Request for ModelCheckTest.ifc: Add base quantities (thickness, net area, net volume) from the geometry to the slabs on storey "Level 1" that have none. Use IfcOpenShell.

First a look at what the model holds.

```python
import ifcopenshell
import ifcopenshell.util.element
import ifcopenshell.util.unit

model = ifcopenshell.open("ModelCheckTest.ifc")
print(model.schema)
for unit_type in ("LENGTHUNIT", "AREAUNIT", "VOLUMEUNIT"):
    print(unit_type, ifcopenshell.util.unit.calculate_unit_scale(model, unit_type))
storey = next(s for s in model.by_type("IfcBuildingStorey") if s.Name == "Level 1")
slabs = [e for e in ifcopenshell.util.element.get_decomposition(storey) if e.is_a("IfcSlab")]
for e in sorted(slabs, key=lambda e: e.id()):
    print(e.id(), e.is_a(), e.Name, list(ifcopenshell.util.element.get_psets(e, qtos_only=True)), sep=" | ")
```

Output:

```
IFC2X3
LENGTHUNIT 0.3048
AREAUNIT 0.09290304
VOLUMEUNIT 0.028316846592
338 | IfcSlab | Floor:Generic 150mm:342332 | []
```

```python
import ifcopenshell
import ifcopenshell.api.pset
import ifcopenshell.geom
import ifcopenshell.util.element
import ifcopenshell.util.shape
import ifcopenshell.util.unit

model = ifcopenshell.open("ModelCheckTest.ifc")
unit_scale = ifcopenshell.util.unit.calculate_unit_scale(model)
area_scale = ifcopenshell.util.unit.calculate_unit_scale(model, "AREAUNIT")
volume_scale = ifcopenshell.util.unit.calculate_unit_scale(model, "VOLUMEUNIT")
settings = ifcopenshell.geom.settings()

storey = next(s for s in model.by_type("IfcBuildingStorey") if s.Name == "Level 1")
slabs = [e for e in ifcopenshell.util.element.get_decomposition(storey) if e.is_a("IfcSlab")]

for e in sorted(slabs, key=lambda e: e.id()):
    if ifcopenshell.util.element.get_psets(e, qtos_only=True, should_inherit=False):
        continue
    # Geometry comes back in metres, in the element's own axes.
    shape = ifcopenshell.geom.create_shape(settings, e)
    values = {
        "Width": ifcopenshell.util.shape.get_z(shape.geometry) / unit_scale,
        "NetArea": ifcopenshell.util.shape.get_footprint_area(shape.geometry) / area_scale,
        "NetVolume": ifcopenshell.util.shape.get_volume(shape.geometry) / volume_scale,
    }
    qto = ifcopenshell.api.pset.add_qto(model, product=e, name="BaseQuantities")
    ifcopenshell.api.pset.edit_qto(model, qto=qto, properties=values)
    print(e.id(), {k: round(v, 3) for k, v in values.items()})

model.write("ModelCheckTest_edited.ifc")
```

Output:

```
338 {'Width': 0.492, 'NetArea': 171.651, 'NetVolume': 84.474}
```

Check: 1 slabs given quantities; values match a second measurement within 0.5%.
